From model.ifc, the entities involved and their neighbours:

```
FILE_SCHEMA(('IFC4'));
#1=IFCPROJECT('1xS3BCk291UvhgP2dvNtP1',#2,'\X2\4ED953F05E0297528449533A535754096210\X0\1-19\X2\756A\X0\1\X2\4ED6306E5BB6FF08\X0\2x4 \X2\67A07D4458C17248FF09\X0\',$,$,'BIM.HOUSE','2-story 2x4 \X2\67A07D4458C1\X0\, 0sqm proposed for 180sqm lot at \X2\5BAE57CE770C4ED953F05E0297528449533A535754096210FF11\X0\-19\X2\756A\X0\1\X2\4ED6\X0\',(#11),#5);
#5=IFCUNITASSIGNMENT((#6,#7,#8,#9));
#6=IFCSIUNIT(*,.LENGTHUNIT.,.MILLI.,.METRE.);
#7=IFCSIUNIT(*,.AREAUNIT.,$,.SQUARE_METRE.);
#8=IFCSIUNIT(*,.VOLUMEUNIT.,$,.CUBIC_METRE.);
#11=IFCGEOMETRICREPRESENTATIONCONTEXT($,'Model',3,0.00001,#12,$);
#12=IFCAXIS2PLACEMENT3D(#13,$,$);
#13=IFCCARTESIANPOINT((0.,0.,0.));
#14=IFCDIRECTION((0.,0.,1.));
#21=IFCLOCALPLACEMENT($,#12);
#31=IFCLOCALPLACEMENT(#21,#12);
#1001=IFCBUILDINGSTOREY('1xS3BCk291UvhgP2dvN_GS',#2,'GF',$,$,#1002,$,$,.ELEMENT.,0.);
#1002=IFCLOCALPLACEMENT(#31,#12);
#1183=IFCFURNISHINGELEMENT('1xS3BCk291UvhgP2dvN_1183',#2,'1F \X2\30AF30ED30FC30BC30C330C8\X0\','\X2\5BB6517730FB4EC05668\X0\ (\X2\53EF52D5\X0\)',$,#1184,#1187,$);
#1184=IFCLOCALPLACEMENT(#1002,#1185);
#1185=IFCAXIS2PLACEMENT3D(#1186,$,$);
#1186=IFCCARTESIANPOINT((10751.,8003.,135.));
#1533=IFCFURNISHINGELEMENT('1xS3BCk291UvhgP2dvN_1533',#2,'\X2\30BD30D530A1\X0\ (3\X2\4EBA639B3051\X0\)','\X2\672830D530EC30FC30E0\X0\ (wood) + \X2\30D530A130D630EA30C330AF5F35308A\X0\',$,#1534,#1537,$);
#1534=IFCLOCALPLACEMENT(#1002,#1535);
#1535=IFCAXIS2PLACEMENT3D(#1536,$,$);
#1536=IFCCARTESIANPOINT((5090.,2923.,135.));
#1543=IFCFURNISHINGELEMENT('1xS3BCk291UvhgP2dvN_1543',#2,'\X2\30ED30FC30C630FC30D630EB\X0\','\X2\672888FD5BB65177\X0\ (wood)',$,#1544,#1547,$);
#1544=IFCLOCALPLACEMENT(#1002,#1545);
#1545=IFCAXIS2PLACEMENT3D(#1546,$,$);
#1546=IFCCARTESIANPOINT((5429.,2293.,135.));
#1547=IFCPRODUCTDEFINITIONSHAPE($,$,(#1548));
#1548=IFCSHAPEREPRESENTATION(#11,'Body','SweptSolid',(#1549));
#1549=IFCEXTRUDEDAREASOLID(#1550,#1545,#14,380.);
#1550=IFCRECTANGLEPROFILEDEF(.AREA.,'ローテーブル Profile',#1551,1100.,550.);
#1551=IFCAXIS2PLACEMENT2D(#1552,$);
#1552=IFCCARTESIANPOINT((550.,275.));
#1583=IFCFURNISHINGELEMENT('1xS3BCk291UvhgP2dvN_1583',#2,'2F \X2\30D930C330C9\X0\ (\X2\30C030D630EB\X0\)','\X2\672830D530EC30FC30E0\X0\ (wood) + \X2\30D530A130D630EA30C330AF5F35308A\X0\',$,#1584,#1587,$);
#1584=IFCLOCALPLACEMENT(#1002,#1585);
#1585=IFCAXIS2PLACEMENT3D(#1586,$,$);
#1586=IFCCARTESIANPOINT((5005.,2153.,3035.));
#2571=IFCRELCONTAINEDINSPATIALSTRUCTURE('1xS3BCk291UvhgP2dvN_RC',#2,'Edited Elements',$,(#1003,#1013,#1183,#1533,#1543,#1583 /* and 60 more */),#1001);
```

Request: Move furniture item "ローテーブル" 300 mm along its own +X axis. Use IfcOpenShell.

```python
import ifcopenshell
import ifcopenshell.api.geometry
import ifcopenshell.util.placement

model = ifcopenshell.open("model.ifc")

item = model.by_id(1543)
matrix = ifcopenshell.util.placement.get_local_placement(item.ObjectPlacement)
matrix[:3, 3] += matrix[:3, 0] * 300.0
ifcopenshell.api.geometry.edit_object_placement(model, product=item, matrix=matrix, is_si=False)

print(ifcopenshell.util.placement.get_local_placement(item.ObjectPlacement).round(3) + 0.0)

model.write("model_v2.ifc")
```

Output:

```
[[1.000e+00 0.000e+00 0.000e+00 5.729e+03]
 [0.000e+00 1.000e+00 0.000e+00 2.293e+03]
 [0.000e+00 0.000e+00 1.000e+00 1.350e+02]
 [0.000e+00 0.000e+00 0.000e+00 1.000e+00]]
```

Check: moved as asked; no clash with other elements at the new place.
